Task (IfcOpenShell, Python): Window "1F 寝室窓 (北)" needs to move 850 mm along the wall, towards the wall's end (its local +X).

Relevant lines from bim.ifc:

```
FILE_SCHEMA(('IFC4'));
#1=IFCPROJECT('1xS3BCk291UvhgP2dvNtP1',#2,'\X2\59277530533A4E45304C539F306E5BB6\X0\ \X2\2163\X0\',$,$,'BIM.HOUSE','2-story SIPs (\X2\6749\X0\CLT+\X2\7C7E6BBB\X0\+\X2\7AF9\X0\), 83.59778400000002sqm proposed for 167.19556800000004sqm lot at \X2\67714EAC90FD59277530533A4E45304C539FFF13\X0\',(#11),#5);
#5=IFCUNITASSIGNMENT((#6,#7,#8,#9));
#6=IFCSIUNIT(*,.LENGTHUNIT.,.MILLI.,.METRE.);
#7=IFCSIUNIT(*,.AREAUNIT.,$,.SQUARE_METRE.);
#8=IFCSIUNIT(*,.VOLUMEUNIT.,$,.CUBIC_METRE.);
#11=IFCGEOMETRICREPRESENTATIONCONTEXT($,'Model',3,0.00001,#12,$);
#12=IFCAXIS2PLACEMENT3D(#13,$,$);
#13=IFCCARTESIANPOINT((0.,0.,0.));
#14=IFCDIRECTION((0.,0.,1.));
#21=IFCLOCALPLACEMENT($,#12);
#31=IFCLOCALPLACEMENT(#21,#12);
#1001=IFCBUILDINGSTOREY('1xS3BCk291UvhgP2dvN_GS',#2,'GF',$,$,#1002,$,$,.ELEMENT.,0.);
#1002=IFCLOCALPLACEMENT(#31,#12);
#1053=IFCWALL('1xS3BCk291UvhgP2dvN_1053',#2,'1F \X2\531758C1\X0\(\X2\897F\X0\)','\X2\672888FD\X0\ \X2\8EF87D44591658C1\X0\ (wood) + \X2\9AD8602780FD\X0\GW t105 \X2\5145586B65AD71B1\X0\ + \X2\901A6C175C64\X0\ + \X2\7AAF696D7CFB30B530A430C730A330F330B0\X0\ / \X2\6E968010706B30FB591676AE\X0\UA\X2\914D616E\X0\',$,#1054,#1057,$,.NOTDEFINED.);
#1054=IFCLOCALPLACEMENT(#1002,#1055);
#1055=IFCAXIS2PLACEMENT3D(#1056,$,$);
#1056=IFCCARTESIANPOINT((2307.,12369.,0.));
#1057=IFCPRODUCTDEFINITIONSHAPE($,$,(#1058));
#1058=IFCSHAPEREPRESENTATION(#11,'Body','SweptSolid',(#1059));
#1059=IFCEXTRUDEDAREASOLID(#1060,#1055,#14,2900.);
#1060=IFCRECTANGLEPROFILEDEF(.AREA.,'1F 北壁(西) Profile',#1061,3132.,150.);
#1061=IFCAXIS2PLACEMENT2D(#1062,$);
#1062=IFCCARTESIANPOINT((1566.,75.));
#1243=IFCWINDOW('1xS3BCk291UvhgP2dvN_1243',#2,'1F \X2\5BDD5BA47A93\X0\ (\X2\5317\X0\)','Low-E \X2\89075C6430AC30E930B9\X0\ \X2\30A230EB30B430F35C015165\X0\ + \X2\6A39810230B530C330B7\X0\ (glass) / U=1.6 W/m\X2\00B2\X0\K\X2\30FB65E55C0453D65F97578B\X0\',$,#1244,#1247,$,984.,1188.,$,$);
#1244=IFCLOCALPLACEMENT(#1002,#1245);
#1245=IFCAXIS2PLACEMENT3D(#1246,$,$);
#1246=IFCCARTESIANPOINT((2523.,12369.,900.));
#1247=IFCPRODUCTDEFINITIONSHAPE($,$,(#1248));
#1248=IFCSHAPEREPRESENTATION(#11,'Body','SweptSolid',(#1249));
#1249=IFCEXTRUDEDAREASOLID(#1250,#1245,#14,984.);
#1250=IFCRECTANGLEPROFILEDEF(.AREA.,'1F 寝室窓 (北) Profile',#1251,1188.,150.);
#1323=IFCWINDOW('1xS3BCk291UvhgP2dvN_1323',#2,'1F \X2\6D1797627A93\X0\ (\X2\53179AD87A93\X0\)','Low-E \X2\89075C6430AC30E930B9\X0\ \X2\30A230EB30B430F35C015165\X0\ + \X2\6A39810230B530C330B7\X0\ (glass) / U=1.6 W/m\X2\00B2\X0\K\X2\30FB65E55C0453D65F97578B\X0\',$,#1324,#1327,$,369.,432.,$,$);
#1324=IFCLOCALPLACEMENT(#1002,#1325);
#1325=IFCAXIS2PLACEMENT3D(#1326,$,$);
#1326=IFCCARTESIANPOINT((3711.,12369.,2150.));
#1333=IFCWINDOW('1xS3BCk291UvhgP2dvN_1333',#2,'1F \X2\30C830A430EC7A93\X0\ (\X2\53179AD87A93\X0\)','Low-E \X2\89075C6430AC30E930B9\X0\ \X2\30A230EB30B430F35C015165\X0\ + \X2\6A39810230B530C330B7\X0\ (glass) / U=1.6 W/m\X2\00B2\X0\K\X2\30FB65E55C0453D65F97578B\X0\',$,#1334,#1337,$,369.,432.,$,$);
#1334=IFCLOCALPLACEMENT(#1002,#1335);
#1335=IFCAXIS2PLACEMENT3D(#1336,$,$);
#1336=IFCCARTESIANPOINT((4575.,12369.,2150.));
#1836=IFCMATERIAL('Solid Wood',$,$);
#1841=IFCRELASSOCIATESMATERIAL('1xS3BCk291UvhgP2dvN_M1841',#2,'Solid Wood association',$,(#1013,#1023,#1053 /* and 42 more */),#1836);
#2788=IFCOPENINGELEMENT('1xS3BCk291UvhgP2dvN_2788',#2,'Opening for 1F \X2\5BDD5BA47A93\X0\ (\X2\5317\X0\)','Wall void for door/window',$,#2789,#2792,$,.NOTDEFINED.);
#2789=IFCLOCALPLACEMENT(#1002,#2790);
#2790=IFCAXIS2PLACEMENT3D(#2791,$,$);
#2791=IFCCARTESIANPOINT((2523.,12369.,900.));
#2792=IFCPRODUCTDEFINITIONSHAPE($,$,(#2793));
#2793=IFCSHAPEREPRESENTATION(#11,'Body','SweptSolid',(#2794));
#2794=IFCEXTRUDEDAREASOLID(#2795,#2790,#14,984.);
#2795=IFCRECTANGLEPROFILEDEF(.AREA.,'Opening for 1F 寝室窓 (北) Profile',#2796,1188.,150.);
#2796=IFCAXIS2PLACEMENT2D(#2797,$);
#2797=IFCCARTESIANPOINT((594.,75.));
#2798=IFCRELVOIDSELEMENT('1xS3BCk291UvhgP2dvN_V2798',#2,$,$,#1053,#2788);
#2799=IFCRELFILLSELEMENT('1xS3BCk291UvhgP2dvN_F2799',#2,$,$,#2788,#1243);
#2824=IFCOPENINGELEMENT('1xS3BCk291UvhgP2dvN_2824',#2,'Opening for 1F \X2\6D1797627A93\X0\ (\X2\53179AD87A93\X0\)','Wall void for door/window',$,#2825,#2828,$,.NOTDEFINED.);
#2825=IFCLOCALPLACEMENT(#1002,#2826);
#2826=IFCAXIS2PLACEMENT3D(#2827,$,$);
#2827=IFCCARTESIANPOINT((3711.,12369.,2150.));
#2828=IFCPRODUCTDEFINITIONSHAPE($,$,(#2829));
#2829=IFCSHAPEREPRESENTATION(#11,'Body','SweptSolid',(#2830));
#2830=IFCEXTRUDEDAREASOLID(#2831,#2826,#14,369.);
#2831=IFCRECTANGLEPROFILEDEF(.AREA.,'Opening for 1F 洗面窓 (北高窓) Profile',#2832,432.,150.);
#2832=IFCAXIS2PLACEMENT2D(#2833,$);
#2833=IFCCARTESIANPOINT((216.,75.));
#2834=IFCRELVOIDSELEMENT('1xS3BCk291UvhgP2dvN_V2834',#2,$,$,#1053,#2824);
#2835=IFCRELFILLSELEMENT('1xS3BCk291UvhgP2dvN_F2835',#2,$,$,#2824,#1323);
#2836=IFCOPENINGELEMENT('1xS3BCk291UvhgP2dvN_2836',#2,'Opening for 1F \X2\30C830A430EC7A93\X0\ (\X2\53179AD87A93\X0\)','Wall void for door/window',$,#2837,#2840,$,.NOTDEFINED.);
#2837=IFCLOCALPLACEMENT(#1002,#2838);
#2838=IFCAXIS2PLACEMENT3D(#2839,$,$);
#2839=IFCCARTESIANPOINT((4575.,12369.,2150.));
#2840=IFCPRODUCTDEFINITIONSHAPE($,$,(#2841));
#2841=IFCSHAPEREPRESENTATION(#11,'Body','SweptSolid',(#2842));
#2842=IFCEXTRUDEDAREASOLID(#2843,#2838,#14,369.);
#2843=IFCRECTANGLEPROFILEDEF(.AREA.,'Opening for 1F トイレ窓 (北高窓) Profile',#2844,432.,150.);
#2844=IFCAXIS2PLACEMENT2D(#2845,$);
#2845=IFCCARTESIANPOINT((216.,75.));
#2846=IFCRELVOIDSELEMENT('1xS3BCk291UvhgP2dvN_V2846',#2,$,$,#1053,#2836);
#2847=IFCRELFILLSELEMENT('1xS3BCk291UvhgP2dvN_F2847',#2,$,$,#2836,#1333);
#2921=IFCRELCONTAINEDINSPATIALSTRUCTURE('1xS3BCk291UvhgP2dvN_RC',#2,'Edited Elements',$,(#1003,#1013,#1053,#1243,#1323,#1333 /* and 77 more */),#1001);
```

```python
import ifcopenshell
import ifcopenshell.api.geometry
import ifcopenshell.util.placement
import ifcopenshell.util.unit

model = ifcopenshell.open("bim.ifc")
unit_scale = ifcopenshell.util.unit.calculate_unit_scale(model)

window = model.by_guid("1xS3BCk291UvhgP2dvN_1243")
opening = window.FillsVoids[0].RelatingOpeningElement
wall = opening.VoidsElements[0].RelatingBuildingElement

wall_matrix = ifcopenshell.util.placement.get_local_placement(wall.ObjectPlacement)
shift = wall_matrix[:3, 0] * 0.85 / unit_scale
before = ifcopenshell.util.placement.get_local_placement(window.ObjectPlacement)[:3, 3].copy()

# The window is not placed relative to its opening, so move both.
for product in (opening, window):
    matrix = ifcopenshell.util.placement.get_local_placement(product.ObjectPlacement)
    matrix[:3, 3] += shift
    ifcopenshell.api.geometry.edit_object_placement(model, product=product, matrix=matrix, is_si=False)

after = ifcopenshell.util.placement.get_local_placement(window.ObjectPlacement)[:3, 3]
print("window moved by", (after - before).round(3) + 0.0)

model.write("bim_updated.ifc")
```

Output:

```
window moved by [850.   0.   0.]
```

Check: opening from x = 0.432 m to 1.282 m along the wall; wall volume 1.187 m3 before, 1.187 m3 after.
